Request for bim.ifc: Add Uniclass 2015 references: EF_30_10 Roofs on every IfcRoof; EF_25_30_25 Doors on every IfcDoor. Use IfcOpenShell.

First a look at what the model holds.

```python
import ifcopenshell

model = ifcopenshell.open("bim.ifc")
print(model.schema)
print("classifications:", [c.Name for c in model.by_type("IfcClassification")])
for ifc_class in ("IfcDoor", "IfcRoof", "IfcStair", "IfcWall", "IfcWindow"):
    print(ifc_class, len(model.by_type(ifc_class)))
```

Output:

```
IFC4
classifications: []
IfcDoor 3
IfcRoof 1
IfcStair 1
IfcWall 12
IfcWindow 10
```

```python
import ifcopenshell
import ifcopenshell.api.classification

model = ifcopenshell.open("bim.ifc")

system = ifcopenshell.api.classification.add_classification(model, classification="Uniclass 2015")

codes = {
    "IfcRoof": ("EF_30_10", "Roofs"),
    "IfcDoor": ("EF_25_30_25", "Doors"),
}
for ifc_class, (code, name) in codes.items():
    products = model.by_type(ifc_class)
    ifcopenshell.api.classification.add_reference(
        model, products=products, classification=system, identification=code, name=name
    )
    print(code, len(products))

model.write("bim_edited.ifc")
```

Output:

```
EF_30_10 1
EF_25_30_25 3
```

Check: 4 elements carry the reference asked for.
